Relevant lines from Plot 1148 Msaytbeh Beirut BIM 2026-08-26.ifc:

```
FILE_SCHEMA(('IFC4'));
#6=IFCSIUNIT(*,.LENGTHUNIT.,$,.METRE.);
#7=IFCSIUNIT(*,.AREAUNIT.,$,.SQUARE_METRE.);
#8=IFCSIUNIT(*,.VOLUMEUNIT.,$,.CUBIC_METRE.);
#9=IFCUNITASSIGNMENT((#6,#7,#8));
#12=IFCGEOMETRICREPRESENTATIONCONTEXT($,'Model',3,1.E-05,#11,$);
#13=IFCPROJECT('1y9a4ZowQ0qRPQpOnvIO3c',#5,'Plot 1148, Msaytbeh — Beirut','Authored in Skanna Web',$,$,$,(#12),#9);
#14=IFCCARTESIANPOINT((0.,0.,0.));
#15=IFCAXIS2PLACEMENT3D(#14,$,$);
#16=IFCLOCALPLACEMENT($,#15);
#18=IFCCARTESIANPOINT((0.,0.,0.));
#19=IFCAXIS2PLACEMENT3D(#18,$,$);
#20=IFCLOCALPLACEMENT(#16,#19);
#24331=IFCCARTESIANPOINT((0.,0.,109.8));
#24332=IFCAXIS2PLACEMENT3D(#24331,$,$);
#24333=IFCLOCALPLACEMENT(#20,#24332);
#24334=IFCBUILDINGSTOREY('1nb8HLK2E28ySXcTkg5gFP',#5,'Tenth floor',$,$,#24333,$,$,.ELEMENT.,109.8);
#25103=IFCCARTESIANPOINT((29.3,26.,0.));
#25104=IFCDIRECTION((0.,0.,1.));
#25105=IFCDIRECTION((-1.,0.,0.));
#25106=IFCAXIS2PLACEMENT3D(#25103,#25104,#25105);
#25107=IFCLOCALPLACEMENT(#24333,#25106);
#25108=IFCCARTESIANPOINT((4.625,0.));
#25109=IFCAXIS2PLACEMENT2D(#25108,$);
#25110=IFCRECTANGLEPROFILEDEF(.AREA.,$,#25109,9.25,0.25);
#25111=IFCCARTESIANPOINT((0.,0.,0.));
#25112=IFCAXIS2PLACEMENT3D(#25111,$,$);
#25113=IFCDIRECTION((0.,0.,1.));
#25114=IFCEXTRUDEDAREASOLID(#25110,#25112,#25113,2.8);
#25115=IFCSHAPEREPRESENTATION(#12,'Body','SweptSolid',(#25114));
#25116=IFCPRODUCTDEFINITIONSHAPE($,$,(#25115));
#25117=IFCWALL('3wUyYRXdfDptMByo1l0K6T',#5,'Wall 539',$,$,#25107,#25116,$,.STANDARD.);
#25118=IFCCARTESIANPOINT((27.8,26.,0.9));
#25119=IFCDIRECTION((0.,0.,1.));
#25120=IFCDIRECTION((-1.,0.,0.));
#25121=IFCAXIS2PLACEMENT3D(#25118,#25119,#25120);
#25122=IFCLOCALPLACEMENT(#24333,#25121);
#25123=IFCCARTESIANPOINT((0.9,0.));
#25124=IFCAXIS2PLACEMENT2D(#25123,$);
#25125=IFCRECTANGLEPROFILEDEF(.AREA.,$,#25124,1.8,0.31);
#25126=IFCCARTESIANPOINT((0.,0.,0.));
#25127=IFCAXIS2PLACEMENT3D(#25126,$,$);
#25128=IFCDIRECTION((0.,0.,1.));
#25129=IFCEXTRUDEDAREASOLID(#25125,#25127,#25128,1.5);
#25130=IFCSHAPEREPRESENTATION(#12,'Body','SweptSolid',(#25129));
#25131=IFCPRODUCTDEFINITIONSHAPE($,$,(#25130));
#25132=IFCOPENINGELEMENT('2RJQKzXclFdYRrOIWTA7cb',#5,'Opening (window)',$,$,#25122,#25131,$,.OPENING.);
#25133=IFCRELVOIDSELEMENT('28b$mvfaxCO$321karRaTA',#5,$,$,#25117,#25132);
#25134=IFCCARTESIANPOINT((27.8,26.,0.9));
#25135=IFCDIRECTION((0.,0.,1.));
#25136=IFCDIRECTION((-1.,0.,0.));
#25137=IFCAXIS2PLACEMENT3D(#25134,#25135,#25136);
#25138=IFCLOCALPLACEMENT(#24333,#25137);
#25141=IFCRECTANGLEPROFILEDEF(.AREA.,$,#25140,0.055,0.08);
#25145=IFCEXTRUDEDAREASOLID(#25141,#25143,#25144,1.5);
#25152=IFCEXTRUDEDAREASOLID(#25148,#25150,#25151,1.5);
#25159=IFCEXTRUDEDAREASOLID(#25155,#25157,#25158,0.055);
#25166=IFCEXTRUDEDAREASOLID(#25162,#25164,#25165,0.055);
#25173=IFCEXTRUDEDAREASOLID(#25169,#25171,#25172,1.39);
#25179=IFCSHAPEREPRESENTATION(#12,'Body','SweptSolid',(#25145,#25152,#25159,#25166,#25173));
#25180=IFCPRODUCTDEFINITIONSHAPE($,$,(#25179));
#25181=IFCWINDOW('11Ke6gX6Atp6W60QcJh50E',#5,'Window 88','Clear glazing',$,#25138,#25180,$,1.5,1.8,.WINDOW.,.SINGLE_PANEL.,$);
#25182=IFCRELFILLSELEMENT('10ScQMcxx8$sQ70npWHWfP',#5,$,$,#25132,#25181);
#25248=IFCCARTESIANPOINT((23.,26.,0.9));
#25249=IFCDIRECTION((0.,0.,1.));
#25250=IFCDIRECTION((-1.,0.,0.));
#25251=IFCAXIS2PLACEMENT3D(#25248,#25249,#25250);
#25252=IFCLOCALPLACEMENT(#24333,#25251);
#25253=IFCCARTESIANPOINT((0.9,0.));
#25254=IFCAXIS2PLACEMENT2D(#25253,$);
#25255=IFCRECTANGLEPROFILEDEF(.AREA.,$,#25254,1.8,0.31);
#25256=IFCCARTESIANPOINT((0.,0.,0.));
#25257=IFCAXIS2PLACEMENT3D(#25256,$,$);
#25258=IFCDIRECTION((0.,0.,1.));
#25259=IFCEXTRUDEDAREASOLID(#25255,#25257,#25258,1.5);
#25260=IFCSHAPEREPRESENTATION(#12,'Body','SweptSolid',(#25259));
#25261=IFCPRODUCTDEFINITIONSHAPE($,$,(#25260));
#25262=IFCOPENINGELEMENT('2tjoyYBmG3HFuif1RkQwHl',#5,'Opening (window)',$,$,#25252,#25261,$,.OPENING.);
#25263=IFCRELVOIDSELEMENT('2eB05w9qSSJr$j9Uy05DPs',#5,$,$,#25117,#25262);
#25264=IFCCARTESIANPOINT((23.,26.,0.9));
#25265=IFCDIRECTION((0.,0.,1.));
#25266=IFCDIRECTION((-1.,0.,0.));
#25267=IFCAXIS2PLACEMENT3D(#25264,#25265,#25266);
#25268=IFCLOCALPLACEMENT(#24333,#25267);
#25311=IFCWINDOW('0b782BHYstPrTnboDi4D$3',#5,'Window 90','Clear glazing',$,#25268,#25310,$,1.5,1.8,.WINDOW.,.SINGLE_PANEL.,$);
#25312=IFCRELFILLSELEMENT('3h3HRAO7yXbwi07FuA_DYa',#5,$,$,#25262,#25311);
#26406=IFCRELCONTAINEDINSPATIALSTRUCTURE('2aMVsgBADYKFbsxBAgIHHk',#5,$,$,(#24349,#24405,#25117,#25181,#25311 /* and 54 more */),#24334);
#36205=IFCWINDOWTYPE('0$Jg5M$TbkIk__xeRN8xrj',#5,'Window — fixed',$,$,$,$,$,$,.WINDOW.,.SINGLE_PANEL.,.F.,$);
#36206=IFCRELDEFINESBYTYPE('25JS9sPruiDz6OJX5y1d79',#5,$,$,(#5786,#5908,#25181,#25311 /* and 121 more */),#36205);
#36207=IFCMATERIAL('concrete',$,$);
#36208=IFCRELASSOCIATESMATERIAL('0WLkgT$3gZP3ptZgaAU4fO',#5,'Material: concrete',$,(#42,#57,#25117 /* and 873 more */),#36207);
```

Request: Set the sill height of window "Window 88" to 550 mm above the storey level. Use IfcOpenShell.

```python
import numpy as np
import ifcopenshell
import ifcopenshell.api.geometry
import ifcopenshell.geom
import ifcopenshell.util.element
import ifcopenshell.util.placement
import ifcopenshell.util.shape
import ifcopenshell.util.unit

model = ifcopenshell.open("Plot 1148 Msaytbeh Beirut BIM 2026-08-26.ifc")
unit_scale = ifcopenshell.util.unit.calculate_unit_scale(model)

window = model.by_guid("11Ke6gX6Atp6W60QcJh50E")
opening = window.FillsVoids[0].RelatingOpeningElement
storey = ifcopenshell.util.element.get_container(window, ifc_class="IfcBuildingStorey")
level = ifcopenshell.util.placement.get_local_placement(storey.ObjectPlacement)[2, 3]

# The opening's origin need not be at the sill, so measure its lowest point.
shape = ifcopenshell.geom.create_shape(ifcopenshell.geom.settings(), opening)
bottom = ifcopenshell.util.shape.get_shape_bottom_elevation(shape, shape.geometry) / unit_scale
dz = level + 0.55 / unit_scale - bottom

shift = np.array([0.0, 0.0, dz])
# The window is not placed relative to its opening, so move both.
for product in (opening, window):
    matrix = ifcopenshell.util.placement.get_local_placement(product.ObjectPlacement)
    matrix[:3, 3] += shift
    ifcopenshell.api.geometry.edit_object_placement(model, product=product, matrix=matrix, is_si=False)

print(f"moved by {dz * unit_scale:+.3f} m")

model.write("Plot 1148 Msaytbeh Beirut BIM 2026-08-26_edited.ifc")
```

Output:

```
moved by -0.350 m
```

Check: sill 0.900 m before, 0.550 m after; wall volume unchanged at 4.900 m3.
